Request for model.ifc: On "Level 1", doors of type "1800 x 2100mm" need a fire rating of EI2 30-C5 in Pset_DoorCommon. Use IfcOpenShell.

First a look at what the model holds.

```python
import ifcopenshell
import ifcopenshell.util.element

model = ifcopenshell.open("model.ifc")
print(model.schema)
storey = next(s for s in model.by_type("IfcBuildingStorey") if s.Name == "Level 1")
doors = [e for e in ifcopenshell.util.element.get_decomposition(storey) if e.is_a("IfcDoor")]
seen = {}
for e in doors:
    element_type = ifcopenshell.util.element.get_type(e)
    key = (element_type.Name if element_type != e and element_type else None, ifcopenshell.util.element.get_pset(e, "Pset_DoorCommon", "FireRating"))
    seen[key] = seen.get(key, 0) + 1
for (name, value), count in sorted(seen.items(), key=str):
    print(count, "x", name, "|", value)
```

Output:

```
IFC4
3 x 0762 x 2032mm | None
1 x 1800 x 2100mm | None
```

```python
import ifcopenshell
import ifcopenshell.api.pset
import ifcopenshell.util.element

model = ifcopenshell.open("model.ifc")

storey = next(s for s in model.by_type("IfcBuildingStorey") if s.Name == "Level 1")
doors = [e for e in ifcopenshell.util.element.get_decomposition(storey) if e.is_a("IfcDoor")]

count = 0
for e in doors:
    element_type = ifcopenshell.util.element.get_type(e)
    if element_type in (None, e) or element_type.Name != "1800 x 2100mm":
        continue
    # add_pset returns the element's existing set when there is one.
    pset = ifcopenshell.api.pset.add_pset(model, product=e, name="Pset_DoorCommon")
    ifcopenshell.api.pset.edit_pset(model, pset=pset, properties={"FireRating": "EI2 30-C5"})
    count += 1

print(count, "doors updated")

model.write("model_rev.ifc")
```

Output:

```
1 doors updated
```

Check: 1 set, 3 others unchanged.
